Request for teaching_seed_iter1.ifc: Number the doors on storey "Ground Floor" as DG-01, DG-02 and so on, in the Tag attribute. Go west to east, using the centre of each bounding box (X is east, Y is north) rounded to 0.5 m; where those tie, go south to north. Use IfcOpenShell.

First a look at what the model holds.

```python
import ifcopenshell
import ifcopenshell.util.element
import ifcopenshell.util.placement

model = ifcopenshell.open("teaching_seed_iter1.ifc")
print(model.schema)
storey = next(s for s in model.by_type("IfcBuildingStorey") if s.Name == "Ground Floor")
doors = [e for e in ifcopenshell.util.element.get_decomposition(storey) if e.is_a("IfcDoor")]
for e in sorted(doors, key=lambda e: e.id()):
    origin = ifcopenshell.util.placement.get_local_placement(e.ObjectPlacement)[:3, 3]
    print(e.id(), e.Tag, e.Name, origin.round(2) + 0.0, sep=" | ")
```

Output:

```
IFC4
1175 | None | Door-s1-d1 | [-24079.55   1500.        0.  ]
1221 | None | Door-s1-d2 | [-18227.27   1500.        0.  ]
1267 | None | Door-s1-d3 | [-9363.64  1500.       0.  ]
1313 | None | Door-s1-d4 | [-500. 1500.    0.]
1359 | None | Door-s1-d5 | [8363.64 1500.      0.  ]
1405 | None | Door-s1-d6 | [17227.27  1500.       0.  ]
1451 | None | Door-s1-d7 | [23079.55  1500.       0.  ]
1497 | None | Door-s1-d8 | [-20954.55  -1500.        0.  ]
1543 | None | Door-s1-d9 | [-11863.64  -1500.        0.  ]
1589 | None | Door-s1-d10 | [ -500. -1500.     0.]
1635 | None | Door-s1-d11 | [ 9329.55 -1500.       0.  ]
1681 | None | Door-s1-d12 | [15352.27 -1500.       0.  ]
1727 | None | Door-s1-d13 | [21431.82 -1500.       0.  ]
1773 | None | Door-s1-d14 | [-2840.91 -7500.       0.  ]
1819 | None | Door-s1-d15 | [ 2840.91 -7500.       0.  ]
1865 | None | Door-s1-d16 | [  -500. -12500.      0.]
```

```python
import ifcopenshell
import ifcopenshell.geom
import ifcopenshell.util.element
import ifcopenshell.util.shape

model = ifcopenshell.open("teaching_seed_iter1.ifc")
settings = ifcopenshell.geom.settings()
settings.set("use-world-coords", True)


def centre(element):
    shape = ifcopenshell.geom.create_shape(settings, element)
    return ifcopenshell.util.shape.get_bbox_centroid(shape.geometry)


storey = next(s for s in model.by_type("IfcBuildingStorey") if s.Name == "Ground Floor")
doors = [e for e in ifcopenshell.util.element.get_decomposition(storey) if e.is_a("IfcDoor")]

# Insertion points can sit at a corner or the storey origin, so sort by the geometry (in metres).
centres = {e: centre(e) for e in doors}
doors.sort(key=lambda e: (round(centres[e][0] / 0.5), centres[e][1]))

for i, e in enumerate(doors, start=1):
    number = f"DG-{i:02d}"
    e.Tag = number
    print(e.id(), number)

model.write("teaching_seed_iter1-out.ifc")
```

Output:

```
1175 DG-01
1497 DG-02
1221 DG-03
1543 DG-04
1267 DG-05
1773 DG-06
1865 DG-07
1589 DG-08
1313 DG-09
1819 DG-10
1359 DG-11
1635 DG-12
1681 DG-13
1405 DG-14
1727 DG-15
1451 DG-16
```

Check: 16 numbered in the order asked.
